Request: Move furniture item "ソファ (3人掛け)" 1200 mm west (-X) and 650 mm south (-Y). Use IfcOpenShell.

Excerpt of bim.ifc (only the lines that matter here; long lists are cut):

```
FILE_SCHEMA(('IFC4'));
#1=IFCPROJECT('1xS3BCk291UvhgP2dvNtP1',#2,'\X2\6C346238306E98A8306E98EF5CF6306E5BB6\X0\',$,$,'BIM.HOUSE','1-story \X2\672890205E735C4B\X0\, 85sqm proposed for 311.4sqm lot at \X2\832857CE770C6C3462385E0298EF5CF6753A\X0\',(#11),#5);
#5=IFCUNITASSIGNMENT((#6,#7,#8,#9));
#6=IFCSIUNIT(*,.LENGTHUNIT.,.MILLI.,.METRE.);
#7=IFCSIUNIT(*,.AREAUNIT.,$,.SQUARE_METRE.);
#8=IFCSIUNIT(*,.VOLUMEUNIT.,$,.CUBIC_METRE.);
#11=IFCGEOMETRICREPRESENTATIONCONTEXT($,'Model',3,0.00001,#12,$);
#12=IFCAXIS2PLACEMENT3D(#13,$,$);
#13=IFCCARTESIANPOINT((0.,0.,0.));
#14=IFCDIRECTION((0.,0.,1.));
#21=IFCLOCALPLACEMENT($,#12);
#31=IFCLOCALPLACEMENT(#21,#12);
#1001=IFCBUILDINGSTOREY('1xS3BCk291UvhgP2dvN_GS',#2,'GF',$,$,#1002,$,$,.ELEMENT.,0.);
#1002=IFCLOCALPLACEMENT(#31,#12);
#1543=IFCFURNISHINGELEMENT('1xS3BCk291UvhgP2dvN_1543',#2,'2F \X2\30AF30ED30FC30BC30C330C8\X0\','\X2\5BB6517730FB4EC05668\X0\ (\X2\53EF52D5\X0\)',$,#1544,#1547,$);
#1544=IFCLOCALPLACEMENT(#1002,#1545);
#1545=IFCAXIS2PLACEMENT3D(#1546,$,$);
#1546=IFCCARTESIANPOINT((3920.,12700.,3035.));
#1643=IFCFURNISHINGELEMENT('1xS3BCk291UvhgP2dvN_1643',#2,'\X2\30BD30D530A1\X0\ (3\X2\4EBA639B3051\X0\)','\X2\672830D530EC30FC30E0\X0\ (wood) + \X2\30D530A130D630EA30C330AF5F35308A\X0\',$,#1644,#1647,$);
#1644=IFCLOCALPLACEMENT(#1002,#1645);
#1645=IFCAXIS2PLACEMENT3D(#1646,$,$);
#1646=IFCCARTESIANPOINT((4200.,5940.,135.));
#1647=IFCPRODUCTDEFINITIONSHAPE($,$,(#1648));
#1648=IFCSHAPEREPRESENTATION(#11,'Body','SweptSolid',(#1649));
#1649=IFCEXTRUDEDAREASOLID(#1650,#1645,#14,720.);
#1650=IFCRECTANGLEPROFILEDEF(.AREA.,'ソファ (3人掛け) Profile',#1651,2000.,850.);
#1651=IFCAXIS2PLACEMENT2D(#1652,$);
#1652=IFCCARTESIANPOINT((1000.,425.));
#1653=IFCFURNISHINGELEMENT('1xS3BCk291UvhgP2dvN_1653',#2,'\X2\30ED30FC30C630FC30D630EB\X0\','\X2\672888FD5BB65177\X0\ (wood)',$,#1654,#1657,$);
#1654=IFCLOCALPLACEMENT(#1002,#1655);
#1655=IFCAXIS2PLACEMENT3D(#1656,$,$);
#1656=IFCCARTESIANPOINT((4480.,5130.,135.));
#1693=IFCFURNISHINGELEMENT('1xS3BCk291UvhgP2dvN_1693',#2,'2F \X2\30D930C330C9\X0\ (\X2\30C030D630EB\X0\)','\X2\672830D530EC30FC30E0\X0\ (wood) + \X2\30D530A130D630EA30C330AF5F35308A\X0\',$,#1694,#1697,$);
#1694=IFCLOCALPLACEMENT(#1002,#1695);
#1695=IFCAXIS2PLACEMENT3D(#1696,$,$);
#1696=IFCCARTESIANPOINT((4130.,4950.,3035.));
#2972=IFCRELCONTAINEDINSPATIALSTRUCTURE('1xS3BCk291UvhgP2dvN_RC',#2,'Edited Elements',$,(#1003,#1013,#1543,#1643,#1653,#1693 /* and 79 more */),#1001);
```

```python
import ifcopenshell
import ifcopenshell.api.geometry
import ifcopenshell.util.placement
import ifcopenshell.util.unit

model = ifcopenshell.open("bim.ifc")
unit_scale = ifcopenshell.util.unit.calculate_unit_scale(model)

item = model.by_guid("1xS3BCk291UvhgP2dvN_1643")
matrix = ifcopenshell.util.placement.get_local_placement(item.ObjectPlacement)
matrix[0, 3] -= 1.2 / unit_scale
matrix[1, 3] -= 0.65 / unit_scale
ifcopenshell.api.geometry.edit_object_placement(model, product=item, matrix=matrix, is_si=False)

print(ifcopenshell.util.placement.get_local_placement(item.ObjectPlacement).round(3) + 0.0)

model.write("bim_edited.ifc")
```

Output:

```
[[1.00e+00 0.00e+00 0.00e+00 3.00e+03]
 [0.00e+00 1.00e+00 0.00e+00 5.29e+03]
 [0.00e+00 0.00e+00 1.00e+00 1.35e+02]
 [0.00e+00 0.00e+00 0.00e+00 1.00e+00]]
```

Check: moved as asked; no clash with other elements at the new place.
